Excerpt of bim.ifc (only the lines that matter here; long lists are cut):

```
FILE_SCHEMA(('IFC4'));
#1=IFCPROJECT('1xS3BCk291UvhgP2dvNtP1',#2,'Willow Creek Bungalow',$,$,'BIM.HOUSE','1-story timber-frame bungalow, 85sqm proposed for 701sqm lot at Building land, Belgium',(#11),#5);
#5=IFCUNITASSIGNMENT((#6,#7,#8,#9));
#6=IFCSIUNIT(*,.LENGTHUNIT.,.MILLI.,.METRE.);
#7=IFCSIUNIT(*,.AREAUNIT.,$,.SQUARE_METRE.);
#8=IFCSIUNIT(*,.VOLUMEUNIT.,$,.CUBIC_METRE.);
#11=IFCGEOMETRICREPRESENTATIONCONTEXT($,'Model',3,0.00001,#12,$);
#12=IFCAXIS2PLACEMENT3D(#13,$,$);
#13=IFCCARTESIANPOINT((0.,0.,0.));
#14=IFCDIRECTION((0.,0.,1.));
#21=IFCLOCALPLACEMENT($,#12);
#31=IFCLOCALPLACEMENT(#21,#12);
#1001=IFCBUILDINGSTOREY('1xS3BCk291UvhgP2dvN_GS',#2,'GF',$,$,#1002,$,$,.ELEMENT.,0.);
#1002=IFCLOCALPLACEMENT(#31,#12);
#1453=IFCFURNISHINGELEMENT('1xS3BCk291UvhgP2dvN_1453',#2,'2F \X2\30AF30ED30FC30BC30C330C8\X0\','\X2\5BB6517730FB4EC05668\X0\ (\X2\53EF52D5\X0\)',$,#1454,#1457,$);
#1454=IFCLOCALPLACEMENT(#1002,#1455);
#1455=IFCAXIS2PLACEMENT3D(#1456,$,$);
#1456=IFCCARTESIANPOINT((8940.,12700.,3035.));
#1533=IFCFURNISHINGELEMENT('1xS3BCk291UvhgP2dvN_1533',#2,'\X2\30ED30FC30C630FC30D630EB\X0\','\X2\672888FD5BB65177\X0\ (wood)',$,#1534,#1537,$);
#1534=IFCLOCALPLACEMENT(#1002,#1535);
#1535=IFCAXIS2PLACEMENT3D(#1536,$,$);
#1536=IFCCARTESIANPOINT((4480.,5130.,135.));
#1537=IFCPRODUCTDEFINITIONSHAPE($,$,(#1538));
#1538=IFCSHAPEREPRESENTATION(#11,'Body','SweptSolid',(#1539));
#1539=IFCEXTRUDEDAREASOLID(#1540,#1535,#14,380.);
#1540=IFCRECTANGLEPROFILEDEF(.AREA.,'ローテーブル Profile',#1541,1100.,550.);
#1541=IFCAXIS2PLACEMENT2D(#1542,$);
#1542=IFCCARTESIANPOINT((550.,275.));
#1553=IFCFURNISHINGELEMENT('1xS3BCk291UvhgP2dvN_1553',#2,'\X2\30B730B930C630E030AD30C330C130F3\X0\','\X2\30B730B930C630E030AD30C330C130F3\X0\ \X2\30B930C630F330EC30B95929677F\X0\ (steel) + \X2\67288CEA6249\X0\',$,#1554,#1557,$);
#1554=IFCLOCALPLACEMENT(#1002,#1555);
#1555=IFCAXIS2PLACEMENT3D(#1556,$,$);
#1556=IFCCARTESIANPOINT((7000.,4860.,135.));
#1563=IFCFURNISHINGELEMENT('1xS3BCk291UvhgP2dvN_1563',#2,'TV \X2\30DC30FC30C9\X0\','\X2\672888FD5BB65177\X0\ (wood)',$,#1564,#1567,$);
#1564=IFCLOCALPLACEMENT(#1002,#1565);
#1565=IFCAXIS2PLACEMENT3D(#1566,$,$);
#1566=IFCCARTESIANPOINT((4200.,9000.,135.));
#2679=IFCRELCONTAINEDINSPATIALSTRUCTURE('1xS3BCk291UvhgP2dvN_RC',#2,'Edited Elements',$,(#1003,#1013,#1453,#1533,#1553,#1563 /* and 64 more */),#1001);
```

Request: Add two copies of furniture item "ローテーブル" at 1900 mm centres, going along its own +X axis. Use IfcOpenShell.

```python
import ifcopenshell
import ifcopenshell.api.geometry
import ifcopenshell.api.root
import ifcopenshell.util.element
import ifcopenshell.util.placement
import ifcopenshell.util.unit

model = ifcopenshell.open("bim.ifc")
unit_scale = ifcopenshell.util.unit.calculate_unit_scale(model)


def reuse_history(source, copy):
    """copy_class also copies each property set's owner history, people and application; keep the originals."""
    for rel in copy.IsDefinedBy:
        if rel.is_a("IfcRelDefinesByProperties") and (history := rel.RelatingPropertyDefinition.OwnerHistory):
            rel.RelatingPropertyDefinition.OwnerHistory = source.OwnerHistory
            ifcopenshell.util.element.remove_deep2(model, history)


source = model.by_guid("1xS3BCk291UvhgP2dvN_1533")
base = ifcopenshell.util.placement.get_local_placement(source.ObjectPlacement)
step = base[:3, 0] * 1.9 / unit_scale

for i in range(1, 3):
    copy = ifcopenshell.api.root.copy_class(model, product=source)
    copy.Representation = ifcopenshell.util.element.copy_deep(
        model, source.Representation, exclude=["IfcGeometricRepresentationContext", "IfcRepresentationMap"]
    )
    reuse_history(source, copy)
    matrix = base.copy()
    matrix[:3, 3] += i * step
    print("added at", matrix[:3, 3].round(3) + 0.0)
    ifcopenshell.api.geometry.edit_object_placement(model, product=copy, matrix=matrix, is_si=False)

model.write("bim_edited.ifc")
```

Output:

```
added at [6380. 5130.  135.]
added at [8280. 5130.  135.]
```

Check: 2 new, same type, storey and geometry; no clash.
